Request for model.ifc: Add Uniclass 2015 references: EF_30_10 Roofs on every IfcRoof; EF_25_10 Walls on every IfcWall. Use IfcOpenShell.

First a look at what the model holds.

```python
import ifcopenshell

model = ifcopenshell.open("model.ifc")
print(model.schema)
print("classifications:", [c.Name for c in model.by_type("IfcClassification")])
for ifc_class in ("IfcDoor", "IfcRoof", "IfcStair", "IfcWall", "IfcWindow"):
    print(ifc_class, len(model.by_type(ifc_class)))
```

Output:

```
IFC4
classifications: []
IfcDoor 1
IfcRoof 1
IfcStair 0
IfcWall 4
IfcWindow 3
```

```python
import ifcopenshell
import ifcopenshell.api.classification

model = ifcopenshell.open("model.ifc")

system = ifcopenshell.api.classification.add_classification(model, classification="Uniclass 2015")

codes = {
    "IfcRoof": ("EF_30_10", "Roofs"),
    "IfcWall": ("EF_25_10", "Walls"),
}
for ifc_class, (code, name) in codes.items():
    products = model.by_type(ifc_class)
    ifcopenshell.api.classification.add_reference(
        model, products=products, classification=system, identification=code, name=name
    )
    print(code, len(products))

model.write("model_edited.ifc")
```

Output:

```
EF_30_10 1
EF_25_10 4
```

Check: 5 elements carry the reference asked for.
